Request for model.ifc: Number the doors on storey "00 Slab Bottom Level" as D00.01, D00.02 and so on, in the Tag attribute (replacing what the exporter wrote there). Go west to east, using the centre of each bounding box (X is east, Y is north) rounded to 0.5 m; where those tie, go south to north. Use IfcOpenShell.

First a look at what the model holds.

```python
import ifcopenshell
import ifcopenshell.util.element
import ifcopenshell.util.placement

model = ifcopenshell.open("model.ifc")
print(model.schema)
storey = next(s for s in model.by_type("IfcBuildingStorey") if s.Name == "00 Slab Bottom Level")
doors = [e for e in ifcopenshell.util.element.get_decomposition(storey) if e.is_a("IfcDoor")]
for e in sorted(doors, key=lambda e: e.id()):
    origin = ifcopenshell.util.placement.get_local_placement(e.ObjectPlacement)[:3, 3]
    print(e.id(), e.Tag, e.Name, origin.round(2) + 0.0, sep=" | ")
```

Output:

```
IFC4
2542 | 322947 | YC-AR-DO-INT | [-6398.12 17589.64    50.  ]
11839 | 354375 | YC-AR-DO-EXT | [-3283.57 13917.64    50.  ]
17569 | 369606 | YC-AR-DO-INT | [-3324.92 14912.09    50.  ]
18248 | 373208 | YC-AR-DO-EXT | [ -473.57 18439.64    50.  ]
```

```python
import ifcopenshell
import ifcopenshell.geom
import ifcopenshell.util.element
import ifcopenshell.util.shape

model = ifcopenshell.open("model.ifc")
settings = ifcopenshell.geom.settings()
settings.set("use-world-coords", True)


def centre(element):
    shape = ifcopenshell.geom.create_shape(settings, element)
    return ifcopenshell.util.shape.get_bbox_centroid(shape.geometry)


storey = next(s for s in model.by_type("IfcBuildingStorey") if s.Name == "00 Slab Bottom Level")
doors = [e for e in ifcopenshell.util.element.get_decomposition(storey) if e.is_a("IfcDoor")]

# Insertion points can sit at a corner or the storey origin, so sort by the geometry (in metres).
centres = {e: centre(e) for e in doors}
doors.sort(key=lambda e: (round(centres[e][0] / 0.5), centres[e][1]))

for i, e in enumerate(doors, start=1):
    number = f"D00.{i:02d}"
    e.Tag = number
    print(e.id(), number)

model.write("model_rev.ifc")
```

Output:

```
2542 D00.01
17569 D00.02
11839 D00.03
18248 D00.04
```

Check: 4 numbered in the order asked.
